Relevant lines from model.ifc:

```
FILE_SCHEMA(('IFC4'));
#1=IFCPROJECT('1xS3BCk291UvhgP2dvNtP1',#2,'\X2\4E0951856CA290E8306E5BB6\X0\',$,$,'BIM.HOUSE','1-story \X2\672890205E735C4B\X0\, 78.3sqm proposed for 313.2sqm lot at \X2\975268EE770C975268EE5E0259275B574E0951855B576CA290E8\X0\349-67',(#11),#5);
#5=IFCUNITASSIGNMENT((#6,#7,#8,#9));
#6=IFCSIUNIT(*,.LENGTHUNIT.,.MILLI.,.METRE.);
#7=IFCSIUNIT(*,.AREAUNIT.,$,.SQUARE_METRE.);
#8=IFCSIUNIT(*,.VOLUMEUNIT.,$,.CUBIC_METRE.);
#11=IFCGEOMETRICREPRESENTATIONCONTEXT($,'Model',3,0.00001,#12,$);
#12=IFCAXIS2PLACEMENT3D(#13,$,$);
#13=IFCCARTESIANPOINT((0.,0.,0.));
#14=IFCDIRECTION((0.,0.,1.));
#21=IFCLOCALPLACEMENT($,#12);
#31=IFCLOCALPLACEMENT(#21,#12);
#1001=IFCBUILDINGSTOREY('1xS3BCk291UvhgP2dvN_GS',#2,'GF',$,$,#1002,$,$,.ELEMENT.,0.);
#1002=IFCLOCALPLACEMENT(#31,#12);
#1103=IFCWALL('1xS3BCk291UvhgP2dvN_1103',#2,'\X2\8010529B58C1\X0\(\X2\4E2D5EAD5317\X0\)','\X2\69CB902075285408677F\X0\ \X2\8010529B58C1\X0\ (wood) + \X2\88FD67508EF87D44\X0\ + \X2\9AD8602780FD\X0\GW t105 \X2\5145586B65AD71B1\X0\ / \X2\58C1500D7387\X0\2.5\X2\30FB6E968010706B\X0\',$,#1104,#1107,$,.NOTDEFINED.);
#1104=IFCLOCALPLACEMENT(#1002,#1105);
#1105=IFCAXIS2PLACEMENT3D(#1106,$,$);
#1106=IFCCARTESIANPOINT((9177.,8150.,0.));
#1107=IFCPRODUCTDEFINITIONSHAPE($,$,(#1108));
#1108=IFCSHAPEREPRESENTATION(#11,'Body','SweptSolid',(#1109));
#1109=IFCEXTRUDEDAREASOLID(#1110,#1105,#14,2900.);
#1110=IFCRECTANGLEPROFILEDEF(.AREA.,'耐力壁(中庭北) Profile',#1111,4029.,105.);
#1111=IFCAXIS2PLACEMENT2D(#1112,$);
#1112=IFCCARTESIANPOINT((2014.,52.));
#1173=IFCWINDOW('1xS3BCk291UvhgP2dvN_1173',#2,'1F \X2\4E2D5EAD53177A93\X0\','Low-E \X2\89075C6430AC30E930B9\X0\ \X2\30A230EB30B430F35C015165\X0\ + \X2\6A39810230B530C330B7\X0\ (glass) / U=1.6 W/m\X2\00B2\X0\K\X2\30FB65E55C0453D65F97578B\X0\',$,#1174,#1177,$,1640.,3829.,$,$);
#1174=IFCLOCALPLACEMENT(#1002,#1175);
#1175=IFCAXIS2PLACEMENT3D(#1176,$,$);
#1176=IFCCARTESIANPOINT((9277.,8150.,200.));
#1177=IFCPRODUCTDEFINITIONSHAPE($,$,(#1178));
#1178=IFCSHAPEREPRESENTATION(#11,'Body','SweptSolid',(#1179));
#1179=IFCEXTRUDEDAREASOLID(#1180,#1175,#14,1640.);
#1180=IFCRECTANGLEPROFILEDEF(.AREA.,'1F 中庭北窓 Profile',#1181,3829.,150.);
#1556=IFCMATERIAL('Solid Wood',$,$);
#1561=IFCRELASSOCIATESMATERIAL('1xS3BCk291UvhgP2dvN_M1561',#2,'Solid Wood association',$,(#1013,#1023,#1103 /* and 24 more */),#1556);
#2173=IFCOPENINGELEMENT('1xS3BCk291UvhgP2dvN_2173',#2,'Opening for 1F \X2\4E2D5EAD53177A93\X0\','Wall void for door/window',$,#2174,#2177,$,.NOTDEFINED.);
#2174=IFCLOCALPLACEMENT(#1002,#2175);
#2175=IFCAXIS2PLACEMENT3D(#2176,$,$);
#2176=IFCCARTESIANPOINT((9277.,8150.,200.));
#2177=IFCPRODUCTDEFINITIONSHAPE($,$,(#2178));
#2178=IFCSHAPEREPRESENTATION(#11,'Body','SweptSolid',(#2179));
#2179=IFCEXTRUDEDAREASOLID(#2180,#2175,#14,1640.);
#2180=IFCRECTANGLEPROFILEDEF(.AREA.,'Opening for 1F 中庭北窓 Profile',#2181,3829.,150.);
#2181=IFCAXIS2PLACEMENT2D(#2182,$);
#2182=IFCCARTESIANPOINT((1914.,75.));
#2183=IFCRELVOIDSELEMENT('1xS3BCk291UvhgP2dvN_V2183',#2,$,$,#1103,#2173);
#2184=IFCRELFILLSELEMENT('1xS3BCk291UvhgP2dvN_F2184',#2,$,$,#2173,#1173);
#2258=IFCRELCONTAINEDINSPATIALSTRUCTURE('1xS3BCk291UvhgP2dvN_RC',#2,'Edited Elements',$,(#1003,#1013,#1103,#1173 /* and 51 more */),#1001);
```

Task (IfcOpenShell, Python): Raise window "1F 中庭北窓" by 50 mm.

```python
import numpy as np
import ifcopenshell
import ifcopenshell.api.geometry
import ifcopenshell.util.placement
import ifcopenshell.util.unit

model = ifcopenshell.open("model.ifc")
unit_scale = ifcopenshell.util.unit.calculate_unit_scale(model)

window = model.by_guid("1xS3BCk291UvhgP2dvN_1173")
opening = window.FillsVoids[0].RelatingOpeningElement
dz = 50.0

shift = np.array([0.0, 0.0, dz])
# The window is not placed relative to its opening, so move both.
for product in (opening, window):
    matrix = ifcopenshell.util.placement.get_local_placement(product.ObjectPlacement)
    matrix[:3, 3] += shift
    ifcopenshell.api.geometry.edit_object_placement(model, product=product, matrix=matrix, is_si=False)

print(f"moved by {dz * unit_scale:+.3f} m")

model.write("model-out.ifc")
```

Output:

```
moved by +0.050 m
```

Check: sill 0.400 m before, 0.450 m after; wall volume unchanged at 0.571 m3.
